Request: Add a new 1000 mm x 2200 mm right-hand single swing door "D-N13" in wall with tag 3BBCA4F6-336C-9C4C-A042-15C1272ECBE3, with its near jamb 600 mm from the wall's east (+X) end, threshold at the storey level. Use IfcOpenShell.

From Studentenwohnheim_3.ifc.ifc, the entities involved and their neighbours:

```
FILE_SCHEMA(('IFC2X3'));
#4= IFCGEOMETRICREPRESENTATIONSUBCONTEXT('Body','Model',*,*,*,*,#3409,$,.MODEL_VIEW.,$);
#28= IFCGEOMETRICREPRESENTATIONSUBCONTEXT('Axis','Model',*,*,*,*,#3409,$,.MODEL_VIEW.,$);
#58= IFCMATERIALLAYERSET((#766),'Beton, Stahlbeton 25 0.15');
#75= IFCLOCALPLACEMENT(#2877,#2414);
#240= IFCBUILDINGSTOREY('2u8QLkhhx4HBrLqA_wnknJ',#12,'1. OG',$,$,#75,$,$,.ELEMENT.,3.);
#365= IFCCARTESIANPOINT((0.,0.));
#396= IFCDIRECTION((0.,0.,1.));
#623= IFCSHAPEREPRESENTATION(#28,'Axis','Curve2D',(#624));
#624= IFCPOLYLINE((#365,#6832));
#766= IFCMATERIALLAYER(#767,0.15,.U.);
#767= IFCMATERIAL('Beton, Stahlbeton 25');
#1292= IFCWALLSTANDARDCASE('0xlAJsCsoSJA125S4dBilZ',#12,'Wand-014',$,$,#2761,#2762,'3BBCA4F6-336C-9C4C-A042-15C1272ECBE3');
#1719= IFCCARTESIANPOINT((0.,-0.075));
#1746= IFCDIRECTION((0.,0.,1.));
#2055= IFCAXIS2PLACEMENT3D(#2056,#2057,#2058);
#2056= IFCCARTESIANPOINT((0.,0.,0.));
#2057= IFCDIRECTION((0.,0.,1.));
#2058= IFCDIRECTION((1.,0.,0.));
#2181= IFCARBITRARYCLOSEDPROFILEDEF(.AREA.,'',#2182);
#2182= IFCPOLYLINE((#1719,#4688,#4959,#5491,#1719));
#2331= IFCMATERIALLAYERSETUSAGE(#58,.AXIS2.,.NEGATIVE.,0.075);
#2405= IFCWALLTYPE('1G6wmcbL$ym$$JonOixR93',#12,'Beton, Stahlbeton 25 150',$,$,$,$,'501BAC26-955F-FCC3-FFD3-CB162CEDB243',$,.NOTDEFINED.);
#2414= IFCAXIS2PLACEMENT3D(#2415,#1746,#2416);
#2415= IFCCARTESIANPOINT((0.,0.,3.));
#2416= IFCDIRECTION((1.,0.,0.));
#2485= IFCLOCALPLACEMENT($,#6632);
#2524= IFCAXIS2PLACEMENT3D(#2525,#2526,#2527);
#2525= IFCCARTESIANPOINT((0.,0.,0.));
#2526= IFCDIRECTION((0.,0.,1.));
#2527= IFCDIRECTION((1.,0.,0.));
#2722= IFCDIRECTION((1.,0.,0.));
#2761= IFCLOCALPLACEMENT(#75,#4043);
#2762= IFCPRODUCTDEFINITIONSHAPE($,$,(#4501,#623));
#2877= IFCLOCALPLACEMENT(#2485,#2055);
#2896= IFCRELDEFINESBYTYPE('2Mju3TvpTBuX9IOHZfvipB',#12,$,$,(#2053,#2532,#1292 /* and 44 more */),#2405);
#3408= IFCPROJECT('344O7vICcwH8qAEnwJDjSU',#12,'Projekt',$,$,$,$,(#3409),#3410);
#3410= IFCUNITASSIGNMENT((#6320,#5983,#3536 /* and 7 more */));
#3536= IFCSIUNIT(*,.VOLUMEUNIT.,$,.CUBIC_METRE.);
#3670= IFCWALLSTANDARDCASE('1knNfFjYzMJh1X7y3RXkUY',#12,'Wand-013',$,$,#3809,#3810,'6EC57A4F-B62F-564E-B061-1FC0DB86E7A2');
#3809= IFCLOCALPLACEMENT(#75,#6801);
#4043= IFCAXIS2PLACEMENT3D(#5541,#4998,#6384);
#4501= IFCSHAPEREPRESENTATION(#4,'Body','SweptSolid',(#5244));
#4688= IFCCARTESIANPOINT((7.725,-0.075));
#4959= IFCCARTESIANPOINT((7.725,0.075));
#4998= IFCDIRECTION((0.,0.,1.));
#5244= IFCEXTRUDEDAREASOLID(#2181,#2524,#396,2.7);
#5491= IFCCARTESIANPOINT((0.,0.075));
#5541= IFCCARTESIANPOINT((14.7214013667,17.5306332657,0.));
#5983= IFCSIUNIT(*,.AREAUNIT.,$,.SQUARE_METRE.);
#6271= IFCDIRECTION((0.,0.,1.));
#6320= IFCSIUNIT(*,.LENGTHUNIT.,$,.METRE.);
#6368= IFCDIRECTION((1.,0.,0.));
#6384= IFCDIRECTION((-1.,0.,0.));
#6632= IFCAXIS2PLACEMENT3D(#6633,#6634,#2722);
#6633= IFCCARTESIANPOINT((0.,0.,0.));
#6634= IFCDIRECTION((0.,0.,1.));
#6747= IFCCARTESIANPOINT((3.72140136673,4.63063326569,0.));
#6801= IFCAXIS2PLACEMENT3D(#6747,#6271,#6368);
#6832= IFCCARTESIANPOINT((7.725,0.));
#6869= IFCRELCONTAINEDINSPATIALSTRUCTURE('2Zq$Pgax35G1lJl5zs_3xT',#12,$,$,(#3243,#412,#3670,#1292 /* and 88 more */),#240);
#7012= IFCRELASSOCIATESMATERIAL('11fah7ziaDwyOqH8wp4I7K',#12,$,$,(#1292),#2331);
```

```python
import numpy as np
import ifcopenshell
import ifcopenshell.api.feature
import ifcopenshell.api.geometry
import ifcopenshell.api.root
import ifcopenshell.api.spatial
import ifcopenshell.api.type
import ifcopenshell.geom
import ifcopenshell.util.element
import ifcopenshell.util.placement
import ifcopenshell.util.representation
import ifcopenshell.util.shape
import ifcopenshell.util.unit

model = ifcopenshell.open("Studentenwohnheim_3.ifc.ifc")
unit_scale = ifcopenshell.util.unit.calculate_unit_scale(model)
settings = ifcopenshell.geom.settings()


def volume(element):
    """Net volume in cubic metres, openings subtracted."""
    shape = ifcopenshell.geom.create_shape(settings, element)
    return ifcopenshell.util.shape.get_volume(shape.geometry)


wall = model.by_guid("0xlAJsCsoSJA125S4dBilZ")
storey = ifcopenshell.util.element.get_container(wall, ifc_class="IfcBuildingStorey")
context = ifcopenshell.util.representation.get_context(model, "Model", "Body", "MODEL_VIEW")
before = volume(wall)

width, height, from_end, sill = 1, 2.2, 0.6, 0.0  # metres

# The wall runs along its own X axis, and the end named is its -X end.
wall_shape = ifcopenshell.geom.create_shape(settings, wall)
x, y, z = ifcopenshell.util.shape.get_vertices(wall_shape.geometry).T
start = x.min() + from_end
face, thickness = float(y.min()), float(y.max() - y.min())
wall_matrix = ifcopenshell.util.placement.get_local_placement(wall.ObjectPlacement)
level = ifcopenshell.util.placement.get_local_placement(storey.ObjectPlacement)[2, 3]


def in_wall(x, y):
    """Placement at x, y metres in the wall's axes, at sill height."""
    matrix = wall_matrix.copy()
    matrix[:, 3] = wall_matrix @ np.array([x / unit_scale, y / unit_scale, 0.0, 1.0])
    matrix[2, 3] = level + sill / unit_scale
    return matrix


# Opening: a box that overshoots both wall faces by 50 mm.
opening = ifcopenshell.api.root.create_entity(model, ifc_class="IfcOpeningElement")
box = ifcopenshell.api.geometry.add_wall_representation(
    model, context=context, length=width, height=height, thickness=thickness + 0.1
)
ifcopenshell.api.geometry.assign_representation(model, product=opening, representation=box)
ifcopenshell.api.geometry.edit_object_placement(model, product=opening, matrix=in_wall(start, face - 0.05), is_si=False)
ifcopenshell.api.feature.add_feature(model, feature=opening, element=wall)

door = ifcopenshell.api.root.create_entity(model, ifc_class="IfcDoor", name="D-N13")
door.OverallWidth, door.OverallHeight = width / unit_scale, height / unit_scale
body = ifcopenshell.api.geometry.add_door_representation(
    model,
    context=context,
    overall_width=door.OverallWidth,
    overall_height=door.OverallHeight,
    operation_type="SINGLE_SWING_RIGHT",
    lining_properties={"LiningDepth": thickness / unit_scale, "ThresholdDepth": thickness / unit_scale},
)
ifcopenshell.api.geometry.assign_representation(model, product=door, representation=body)
ifcopenshell.api.spatial.assign_container(model, products=[door], relating_structure=storey)
fills = ifcopenshell.api.feature.add_filling(model, opening=opening, element=door)
fills.OwnerHistory = door.OwnerHistory  # required in IFC2X3

# IFC2X3 keeps the operation on the door style.
style = ifcopenshell.api.root.create_entity(model, ifc_class="IfcDoorStyle", name="D-N13")
style.OperationType, style.ConstructionType = "SINGLE_SWING_RIGHT", "NOTDEFINED"
style.ParameterTakesPrecedence = style.Sizeable = False
ifcopenshell.api.type.assign_type(model, related_objects=[door], relating_type=style)

# The lining spans the wall, so the door starts at the wall face.
ifcopenshell.api.geometry.edit_object_placement(model, product=door, matrix=in_wall(start, face), is_si=False)

after = volume(wall)

print(f"wall volume {before:.3f} -> {after:.3f} m3")

model.write("Studentenwohnheim_3.ifc_edited.ifc")
```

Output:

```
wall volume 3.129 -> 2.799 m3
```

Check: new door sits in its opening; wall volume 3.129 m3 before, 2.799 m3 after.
